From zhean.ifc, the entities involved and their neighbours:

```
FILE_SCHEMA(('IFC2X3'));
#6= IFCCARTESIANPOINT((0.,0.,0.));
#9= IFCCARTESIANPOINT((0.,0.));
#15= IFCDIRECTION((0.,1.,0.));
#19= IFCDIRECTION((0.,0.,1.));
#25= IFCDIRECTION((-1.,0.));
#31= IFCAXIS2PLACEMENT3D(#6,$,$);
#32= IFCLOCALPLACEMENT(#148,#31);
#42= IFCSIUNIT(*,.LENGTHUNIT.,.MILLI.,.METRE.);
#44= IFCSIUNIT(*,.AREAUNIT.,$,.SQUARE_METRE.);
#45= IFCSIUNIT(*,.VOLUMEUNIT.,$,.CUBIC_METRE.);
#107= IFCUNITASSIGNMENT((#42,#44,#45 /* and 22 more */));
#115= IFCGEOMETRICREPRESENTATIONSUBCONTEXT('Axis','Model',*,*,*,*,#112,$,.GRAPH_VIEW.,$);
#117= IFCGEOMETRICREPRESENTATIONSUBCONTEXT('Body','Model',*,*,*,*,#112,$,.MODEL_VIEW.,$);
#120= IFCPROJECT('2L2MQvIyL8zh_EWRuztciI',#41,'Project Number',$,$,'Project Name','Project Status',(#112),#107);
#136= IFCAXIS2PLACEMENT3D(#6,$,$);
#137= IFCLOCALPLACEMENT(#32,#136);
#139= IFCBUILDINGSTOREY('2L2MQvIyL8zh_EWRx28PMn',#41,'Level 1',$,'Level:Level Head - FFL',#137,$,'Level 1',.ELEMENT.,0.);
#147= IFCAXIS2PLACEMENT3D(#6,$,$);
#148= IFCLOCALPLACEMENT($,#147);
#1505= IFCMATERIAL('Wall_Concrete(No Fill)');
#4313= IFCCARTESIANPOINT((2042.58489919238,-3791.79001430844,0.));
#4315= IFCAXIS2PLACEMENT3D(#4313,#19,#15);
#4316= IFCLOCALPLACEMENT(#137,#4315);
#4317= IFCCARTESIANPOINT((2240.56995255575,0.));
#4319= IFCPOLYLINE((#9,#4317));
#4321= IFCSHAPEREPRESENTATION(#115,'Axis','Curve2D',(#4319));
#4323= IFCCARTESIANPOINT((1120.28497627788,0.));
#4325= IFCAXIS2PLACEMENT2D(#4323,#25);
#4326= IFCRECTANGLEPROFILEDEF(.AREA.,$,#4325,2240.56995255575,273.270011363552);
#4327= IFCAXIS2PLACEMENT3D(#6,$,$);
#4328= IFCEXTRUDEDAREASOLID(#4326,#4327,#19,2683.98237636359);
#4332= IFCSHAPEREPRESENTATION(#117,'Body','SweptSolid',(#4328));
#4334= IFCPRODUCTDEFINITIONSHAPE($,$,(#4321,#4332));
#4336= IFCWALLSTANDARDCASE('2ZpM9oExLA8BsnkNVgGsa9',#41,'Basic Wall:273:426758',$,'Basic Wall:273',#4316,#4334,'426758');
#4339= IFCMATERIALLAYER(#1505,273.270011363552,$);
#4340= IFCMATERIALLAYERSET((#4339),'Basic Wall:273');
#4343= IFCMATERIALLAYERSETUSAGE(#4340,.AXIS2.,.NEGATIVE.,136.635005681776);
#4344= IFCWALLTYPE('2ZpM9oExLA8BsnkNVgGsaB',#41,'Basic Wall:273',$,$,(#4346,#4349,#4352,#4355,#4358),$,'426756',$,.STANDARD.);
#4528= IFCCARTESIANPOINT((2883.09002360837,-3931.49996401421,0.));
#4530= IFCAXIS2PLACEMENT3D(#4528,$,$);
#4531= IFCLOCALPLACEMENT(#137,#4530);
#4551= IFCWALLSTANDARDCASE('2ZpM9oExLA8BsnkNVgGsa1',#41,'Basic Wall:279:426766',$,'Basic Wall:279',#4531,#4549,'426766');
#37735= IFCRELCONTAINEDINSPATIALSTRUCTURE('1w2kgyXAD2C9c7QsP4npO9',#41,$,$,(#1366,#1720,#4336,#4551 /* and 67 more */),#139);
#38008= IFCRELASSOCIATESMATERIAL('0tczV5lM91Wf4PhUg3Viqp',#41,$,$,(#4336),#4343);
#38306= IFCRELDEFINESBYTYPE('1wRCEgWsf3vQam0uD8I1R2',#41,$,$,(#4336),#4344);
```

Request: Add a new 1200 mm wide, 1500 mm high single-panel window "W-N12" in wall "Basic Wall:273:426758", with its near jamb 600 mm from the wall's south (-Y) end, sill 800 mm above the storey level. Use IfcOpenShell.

```python
import numpy as np
import ifcopenshell
import ifcopenshell.api.feature
import ifcopenshell.api.geometry
import ifcopenshell.api.root
import ifcopenshell.api.spatial
import ifcopenshell.api.type
import ifcopenshell.geom
import ifcopenshell.util.element
import ifcopenshell.util.placement
import ifcopenshell.util.representation
import ifcopenshell.util.shape
import ifcopenshell.util.unit

model = ifcopenshell.open("zhean.ifc")
unit_scale = ifcopenshell.util.unit.calculate_unit_scale(model)
settings = ifcopenshell.geom.settings()


def volume(element):
    """Net volume in cubic metres, openings subtracted."""
    shape = ifcopenshell.geom.create_shape(settings, element)
    return ifcopenshell.util.shape.get_volume(shape.geometry)


wall = model.by_guid("2ZpM9oExLA8BsnkNVgGsa9")
storey = ifcopenshell.util.element.get_container(wall, ifc_class="IfcBuildingStorey")
context = ifcopenshell.util.representation.get_context(model, "Model", "Body", "MODEL_VIEW")
before = volume(wall)

width, height, from_end, sill = 1.2, 1.5, 0.6, 0.8  # metres

# The wall runs along its own X axis, and the end named is its -X end.
wall_shape = ifcopenshell.geom.create_shape(settings, wall)
x, y, z = ifcopenshell.util.shape.get_vertices(wall_shape.geometry).T
start = x.min() + from_end
face, thickness = float(y.min()), float(y.max() - y.min())
wall_matrix = ifcopenshell.util.placement.get_local_placement(wall.ObjectPlacement)
level = ifcopenshell.util.placement.get_local_placement(storey.ObjectPlacement)[2, 3]


def in_wall(x, y):
    """Placement at x, y metres in the wall's axes, at sill height."""
    matrix = wall_matrix.copy()
    matrix[:, 3] = wall_matrix @ np.array([x / unit_scale, y / unit_scale, 0.0, 1.0])
    matrix[2, 3] = level + sill / unit_scale
    return matrix


# Opening: a box that overshoots both wall faces by 50 mm.
opening = ifcopenshell.api.root.create_entity(model, ifc_class="IfcOpeningElement")
box = ifcopenshell.api.geometry.add_wall_representation(
    model, context=context, length=width, height=height, thickness=thickness + 0.1
)
ifcopenshell.api.geometry.assign_representation(model, product=opening, representation=box)
ifcopenshell.api.geometry.edit_object_placement(model, product=opening, matrix=in_wall(start, face - 0.05), is_si=False)
ifcopenshell.api.feature.add_feature(model, feature=opening, element=wall)

window = ifcopenshell.api.root.create_entity(model, ifc_class="IfcWindow", name="W-N12")
window.OverallWidth, window.OverallHeight = width / unit_scale, height / unit_scale
body = ifcopenshell.api.geometry.add_window_representation(
    model,
    context=context,
    overall_width=window.OverallWidth,
    overall_height=window.OverallHeight,
    partition_type="SINGLE_PANEL",
)
ifcopenshell.api.geometry.assign_representation(model, product=window, representation=body)
ifcopenshell.api.spatial.assign_container(model, products=[window], relating_structure=storey)
fills = ifcopenshell.api.feature.add_filling(model, opening=opening, element=window)
fills.OwnerHistory = window.OwnerHistory  # required in IFC2X3

# IFC2X3 keeps the operation on the window style.
style = ifcopenshell.api.root.create_entity(model, ifc_class="IfcWindowStyle", name="W-N12")
style.OperationType, style.ConstructionType = "SINGLE_PANEL", "NOTDEFINED"
style.ParameterTakesPrecedence = style.Sizeable = False
ifcopenshell.api.type.assign_type(model, related_objects=[window], relating_type=style)

# Centre the window in the wall's thickness.
ifcopenshell.api.geometry.edit_object_placement(model, product=window, matrix=in_wall(start, face), is_si=False)
window_shape = ifcopenshell.geom.create_shape(settings, window)
depth = ifcopenshell.util.shape.get_vertices(window_shape.geometry)[:, 1]
offset = face + thickness / 2 - (depth.min() + depth.max()) / 2
ifcopenshell.api.geometry.edit_object_placement(model, product=window, matrix=in_wall(start, offset), is_si=False)

after = volume(wall)

print(f"wall volume {before:.3f} -> {after:.3f} m3")

model.write("zhean_edited.ifc")
```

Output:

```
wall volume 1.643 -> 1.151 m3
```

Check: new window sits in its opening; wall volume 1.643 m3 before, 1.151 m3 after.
